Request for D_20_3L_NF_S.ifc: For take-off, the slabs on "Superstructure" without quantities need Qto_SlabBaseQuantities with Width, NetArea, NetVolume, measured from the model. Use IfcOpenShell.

First a look at what the model holds.

```python
import ifcopenshell
import ifcopenshell.util.element
import ifcopenshell.util.unit

model = ifcopenshell.open("D_20_3L_NF_S.ifc")
print(model.schema)
for unit_type in ("LENGTHUNIT", "AREAUNIT", "VOLUMEUNIT"):
    print(unit_type, ifcopenshell.util.unit.calculate_unit_scale(model, unit_type))
storey = next(s for s in model.by_type("IfcBuildingStorey") if s.Name == "Superstructure")
slabs = [e for e in ifcopenshell.util.element.get_decomposition(storey) if e.is_a("IfcSlab")]
for e in sorted(slabs, key=lambda e: e.id()):
    print(e.id(), e.is_a(), e.Name, list(ifcopenshell.util.element.get_psets(e, qtos_only=True)), sep=" | ")
```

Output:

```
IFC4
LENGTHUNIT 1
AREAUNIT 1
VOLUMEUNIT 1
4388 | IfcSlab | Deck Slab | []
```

```python
import ifcopenshell
import ifcopenshell.api.pset
import ifcopenshell.geom
import ifcopenshell.util.element
import ifcopenshell.util.shape
import ifcopenshell.util.unit

model = ifcopenshell.open("D_20_3L_NF_S.ifc")
unit_scale = ifcopenshell.util.unit.calculate_unit_scale(model)
area_scale = ifcopenshell.util.unit.calculate_unit_scale(model, "AREAUNIT")
volume_scale = ifcopenshell.util.unit.calculate_unit_scale(model, "VOLUMEUNIT")
settings = ifcopenshell.geom.settings()

storey = next(s for s in model.by_type("IfcBuildingStorey") if s.Name == "Superstructure")
slabs = [e for e in ifcopenshell.util.element.get_decomposition(storey) if e.is_a("IfcSlab")]

for e in sorted(slabs, key=lambda e: e.id()):
    if ifcopenshell.util.element.get_psets(e, qtos_only=True, should_inherit=False):
        continue
    # Geometry comes back in metres, in the element's own axes.
    shape = ifcopenshell.geom.create_shape(settings, e)
    values = {
        "Width": ifcopenshell.util.shape.get_z(shape.geometry) / unit_scale,
        "NetArea": ifcopenshell.util.shape.get_footprint_area(shape.geometry) / area_scale,
        "NetVolume": ifcopenshell.util.shape.get_volume(shape.geometry) / volume_scale,
    }
    qto = ifcopenshell.api.pset.add_qto(model, product=e, name="Qto_SlabBaseQuantities")
    ifcopenshell.api.pset.edit_qto(model, qto=qto, properties=values)
    print(e.id(), {k: round(v, 3) for k, v in values.items()})

model.write("D_20_3L_NF_S_updated.ifc")
```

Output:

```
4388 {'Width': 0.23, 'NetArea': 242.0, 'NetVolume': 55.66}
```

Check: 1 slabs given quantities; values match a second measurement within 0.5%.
